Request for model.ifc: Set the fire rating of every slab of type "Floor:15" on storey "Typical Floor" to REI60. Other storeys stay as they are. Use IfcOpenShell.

First a look at what the model holds.

```python
import ifcopenshell
import ifcopenshell.util.element

model = ifcopenshell.open("model.ifc")
print(model.schema)
storey = next(s for s in model.by_type("IfcBuildingStorey") if s.Name == "Typical Floor")
slabs = [e for e in ifcopenshell.util.element.get_decomposition(storey) if e.is_a("IfcSlab")]
seen = {}
for e in slabs:
    element_type = ifcopenshell.util.element.get_type(e)
    key = (element_type.Name if element_type != e and element_type else None, ifcopenshell.util.element.get_pset(e, "Pset_SlabCommon", "FireRating"))
    seen[key] = seen.get(key, 0) + 1
for (name, value), count in sorted(seen.items(), key=str):
    print(count, "x", name, "|", value)
```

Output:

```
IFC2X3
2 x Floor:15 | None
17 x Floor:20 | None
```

```python
import ifcopenshell
import ifcopenshell.api.pset
import ifcopenshell.util.element

model = ifcopenshell.open("model.ifc")

storey = next(s for s in model.by_type("IfcBuildingStorey") if s.Name == "Typical Floor")
slabs = [e for e in ifcopenshell.util.element.get_decomposition(storey) if e.is_a("IfcSlab")]

count = 0
for e in slabs:
    element_type = ifcopenshell.util.element.get_type(e)
    if element_type in (None, e) or element_type.Name != "Floor:15":
        continue
    # add_pset returns the element's existing set when there is one.
    pset = ifcopenshell.api.pset.add_pset(model, product=e, name="Pset_SlabCommon")
    ifcopenshell.api.pset.edit_pset(model, pset=pset, properties={"FireRating": "REI60"})
    count += 1

print(count, "slabs updated")

model.write("model_updated.ifc")
```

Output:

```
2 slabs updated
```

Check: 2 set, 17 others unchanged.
